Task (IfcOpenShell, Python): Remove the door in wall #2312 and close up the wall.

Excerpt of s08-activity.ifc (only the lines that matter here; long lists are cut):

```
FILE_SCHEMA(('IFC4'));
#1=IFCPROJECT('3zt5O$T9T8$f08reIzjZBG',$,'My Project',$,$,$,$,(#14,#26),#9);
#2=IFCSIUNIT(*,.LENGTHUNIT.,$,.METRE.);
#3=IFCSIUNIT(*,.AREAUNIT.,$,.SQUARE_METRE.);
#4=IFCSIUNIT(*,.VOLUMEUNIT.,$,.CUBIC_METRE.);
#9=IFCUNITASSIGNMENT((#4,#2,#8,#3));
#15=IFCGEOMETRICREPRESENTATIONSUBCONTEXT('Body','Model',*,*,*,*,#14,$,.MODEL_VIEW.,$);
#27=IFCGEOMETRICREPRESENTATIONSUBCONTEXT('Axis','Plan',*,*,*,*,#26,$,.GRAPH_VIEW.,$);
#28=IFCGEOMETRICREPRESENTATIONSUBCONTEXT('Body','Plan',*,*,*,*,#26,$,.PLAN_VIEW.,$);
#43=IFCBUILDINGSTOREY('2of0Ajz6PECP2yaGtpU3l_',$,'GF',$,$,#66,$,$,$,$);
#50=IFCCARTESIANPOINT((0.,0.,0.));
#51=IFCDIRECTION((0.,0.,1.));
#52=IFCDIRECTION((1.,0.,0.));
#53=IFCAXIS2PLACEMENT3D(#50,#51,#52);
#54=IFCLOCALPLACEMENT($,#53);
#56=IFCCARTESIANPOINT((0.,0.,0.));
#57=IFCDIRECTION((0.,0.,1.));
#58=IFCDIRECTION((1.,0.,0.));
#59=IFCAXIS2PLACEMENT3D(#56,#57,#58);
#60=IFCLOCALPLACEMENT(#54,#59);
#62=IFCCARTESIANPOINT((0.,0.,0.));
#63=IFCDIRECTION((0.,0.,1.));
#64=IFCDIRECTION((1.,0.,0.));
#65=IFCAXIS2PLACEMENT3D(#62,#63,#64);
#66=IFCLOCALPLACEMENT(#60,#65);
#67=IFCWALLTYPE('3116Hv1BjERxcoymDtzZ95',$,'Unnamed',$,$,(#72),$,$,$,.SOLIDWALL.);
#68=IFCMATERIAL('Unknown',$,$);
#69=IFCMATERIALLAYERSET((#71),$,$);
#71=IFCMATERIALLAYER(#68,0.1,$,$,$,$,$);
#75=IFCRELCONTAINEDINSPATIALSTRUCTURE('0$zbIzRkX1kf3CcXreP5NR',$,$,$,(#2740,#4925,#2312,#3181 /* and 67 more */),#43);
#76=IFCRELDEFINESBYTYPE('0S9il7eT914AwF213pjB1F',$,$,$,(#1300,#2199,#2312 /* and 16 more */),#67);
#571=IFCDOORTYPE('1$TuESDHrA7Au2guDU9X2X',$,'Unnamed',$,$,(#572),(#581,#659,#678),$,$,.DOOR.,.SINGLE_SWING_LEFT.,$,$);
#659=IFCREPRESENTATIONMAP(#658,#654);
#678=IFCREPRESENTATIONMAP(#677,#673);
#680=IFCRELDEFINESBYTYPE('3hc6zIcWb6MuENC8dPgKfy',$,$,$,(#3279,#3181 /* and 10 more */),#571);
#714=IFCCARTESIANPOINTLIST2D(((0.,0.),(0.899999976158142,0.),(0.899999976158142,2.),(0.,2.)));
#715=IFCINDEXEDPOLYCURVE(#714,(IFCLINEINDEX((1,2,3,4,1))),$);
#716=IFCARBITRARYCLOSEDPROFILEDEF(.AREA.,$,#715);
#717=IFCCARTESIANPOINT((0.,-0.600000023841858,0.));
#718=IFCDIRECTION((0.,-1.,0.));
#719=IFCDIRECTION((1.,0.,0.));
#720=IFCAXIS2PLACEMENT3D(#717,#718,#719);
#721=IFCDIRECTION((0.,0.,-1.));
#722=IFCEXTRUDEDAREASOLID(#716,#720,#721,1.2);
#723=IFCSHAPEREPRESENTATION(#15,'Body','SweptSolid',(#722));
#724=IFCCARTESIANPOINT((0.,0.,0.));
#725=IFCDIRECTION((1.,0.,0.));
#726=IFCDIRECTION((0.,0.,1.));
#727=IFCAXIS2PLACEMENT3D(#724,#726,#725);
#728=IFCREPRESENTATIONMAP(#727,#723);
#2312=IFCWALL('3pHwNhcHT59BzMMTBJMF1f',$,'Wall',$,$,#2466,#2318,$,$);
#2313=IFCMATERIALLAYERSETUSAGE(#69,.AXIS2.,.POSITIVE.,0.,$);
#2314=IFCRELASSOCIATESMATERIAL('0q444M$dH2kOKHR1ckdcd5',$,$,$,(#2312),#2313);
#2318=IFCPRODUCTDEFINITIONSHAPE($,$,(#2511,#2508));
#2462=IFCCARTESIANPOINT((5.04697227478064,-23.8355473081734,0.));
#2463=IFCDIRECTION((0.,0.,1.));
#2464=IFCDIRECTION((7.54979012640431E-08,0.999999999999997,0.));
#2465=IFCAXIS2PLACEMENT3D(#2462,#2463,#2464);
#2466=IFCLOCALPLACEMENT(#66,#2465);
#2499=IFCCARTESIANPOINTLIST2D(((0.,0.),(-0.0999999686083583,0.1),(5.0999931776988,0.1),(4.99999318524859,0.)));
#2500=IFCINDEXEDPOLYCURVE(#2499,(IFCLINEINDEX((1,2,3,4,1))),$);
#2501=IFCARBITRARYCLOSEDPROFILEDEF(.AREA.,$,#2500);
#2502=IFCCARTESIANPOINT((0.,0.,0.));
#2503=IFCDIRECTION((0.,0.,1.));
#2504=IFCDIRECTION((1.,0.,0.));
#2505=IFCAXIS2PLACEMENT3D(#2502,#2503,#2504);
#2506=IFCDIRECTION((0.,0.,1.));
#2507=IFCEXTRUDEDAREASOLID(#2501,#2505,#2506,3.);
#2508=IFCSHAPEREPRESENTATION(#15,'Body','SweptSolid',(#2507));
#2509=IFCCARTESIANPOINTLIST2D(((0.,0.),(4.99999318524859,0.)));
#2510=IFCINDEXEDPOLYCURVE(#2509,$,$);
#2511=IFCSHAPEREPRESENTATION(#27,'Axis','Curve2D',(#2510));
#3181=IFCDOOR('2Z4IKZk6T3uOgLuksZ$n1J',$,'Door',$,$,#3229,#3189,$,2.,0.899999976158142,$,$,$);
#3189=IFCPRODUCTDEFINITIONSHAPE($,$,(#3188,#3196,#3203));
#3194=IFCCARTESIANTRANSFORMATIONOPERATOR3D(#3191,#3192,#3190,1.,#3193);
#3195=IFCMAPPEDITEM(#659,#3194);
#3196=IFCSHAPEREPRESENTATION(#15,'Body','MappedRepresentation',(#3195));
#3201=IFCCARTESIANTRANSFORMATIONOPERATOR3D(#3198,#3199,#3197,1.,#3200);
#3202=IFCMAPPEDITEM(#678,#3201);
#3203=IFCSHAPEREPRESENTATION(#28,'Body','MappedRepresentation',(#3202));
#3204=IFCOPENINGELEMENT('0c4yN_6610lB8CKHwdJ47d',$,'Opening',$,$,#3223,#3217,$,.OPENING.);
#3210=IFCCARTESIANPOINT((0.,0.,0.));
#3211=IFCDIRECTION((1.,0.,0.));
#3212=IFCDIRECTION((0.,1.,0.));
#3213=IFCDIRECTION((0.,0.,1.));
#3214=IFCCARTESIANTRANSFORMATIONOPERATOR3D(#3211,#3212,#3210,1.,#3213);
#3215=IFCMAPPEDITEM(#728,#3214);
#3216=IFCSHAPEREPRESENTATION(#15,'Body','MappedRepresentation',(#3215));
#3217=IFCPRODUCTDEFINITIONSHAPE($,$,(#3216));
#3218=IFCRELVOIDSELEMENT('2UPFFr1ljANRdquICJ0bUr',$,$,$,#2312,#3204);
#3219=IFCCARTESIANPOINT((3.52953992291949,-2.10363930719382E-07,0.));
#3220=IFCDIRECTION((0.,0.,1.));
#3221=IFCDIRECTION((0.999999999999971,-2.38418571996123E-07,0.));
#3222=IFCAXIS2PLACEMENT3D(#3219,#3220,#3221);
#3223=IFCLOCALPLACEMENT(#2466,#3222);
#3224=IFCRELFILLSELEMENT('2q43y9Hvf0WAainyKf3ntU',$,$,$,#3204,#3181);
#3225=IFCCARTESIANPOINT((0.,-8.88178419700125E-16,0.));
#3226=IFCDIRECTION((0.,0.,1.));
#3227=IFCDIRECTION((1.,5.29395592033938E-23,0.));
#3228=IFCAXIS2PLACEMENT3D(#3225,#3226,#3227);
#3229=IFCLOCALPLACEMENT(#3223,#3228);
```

```python
import ifcopenshell
import ifcopenshell.api.feature
import ifcopenshell.api.root
import ifcopenshell.geom
import ifcopenshell.util.shape

model = ifcopenshell.open("s08-activity.ifc")
settings = ifcopenshell.geom.settings()


def volume(element):
    """Net volume in cubic metres, openings subtracted."""
    shape = ifcopenshell.geom.create_shape(settings, element)
    return ifcopenshell.util.shape.get_volume(shape.geometry)


door = model.by_id(3181)
opening = door.FillsVoids[0].RelatingOpeningElement
wall = opening.VoidsElements[0].RelatingBuildingElement
before = volume(wall)

ifcopenshell.api.root.remove_product(model, product=door)
ifcopenshell.api.feature.remove_feature(model, feature=opening)

after = volume(wall)

print(f"wall volume {before:.3f} -> {after:.3f} m3")

model.write("s08-activity_rev.ifc")
```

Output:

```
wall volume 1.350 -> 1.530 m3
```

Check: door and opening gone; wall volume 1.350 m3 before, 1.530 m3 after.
